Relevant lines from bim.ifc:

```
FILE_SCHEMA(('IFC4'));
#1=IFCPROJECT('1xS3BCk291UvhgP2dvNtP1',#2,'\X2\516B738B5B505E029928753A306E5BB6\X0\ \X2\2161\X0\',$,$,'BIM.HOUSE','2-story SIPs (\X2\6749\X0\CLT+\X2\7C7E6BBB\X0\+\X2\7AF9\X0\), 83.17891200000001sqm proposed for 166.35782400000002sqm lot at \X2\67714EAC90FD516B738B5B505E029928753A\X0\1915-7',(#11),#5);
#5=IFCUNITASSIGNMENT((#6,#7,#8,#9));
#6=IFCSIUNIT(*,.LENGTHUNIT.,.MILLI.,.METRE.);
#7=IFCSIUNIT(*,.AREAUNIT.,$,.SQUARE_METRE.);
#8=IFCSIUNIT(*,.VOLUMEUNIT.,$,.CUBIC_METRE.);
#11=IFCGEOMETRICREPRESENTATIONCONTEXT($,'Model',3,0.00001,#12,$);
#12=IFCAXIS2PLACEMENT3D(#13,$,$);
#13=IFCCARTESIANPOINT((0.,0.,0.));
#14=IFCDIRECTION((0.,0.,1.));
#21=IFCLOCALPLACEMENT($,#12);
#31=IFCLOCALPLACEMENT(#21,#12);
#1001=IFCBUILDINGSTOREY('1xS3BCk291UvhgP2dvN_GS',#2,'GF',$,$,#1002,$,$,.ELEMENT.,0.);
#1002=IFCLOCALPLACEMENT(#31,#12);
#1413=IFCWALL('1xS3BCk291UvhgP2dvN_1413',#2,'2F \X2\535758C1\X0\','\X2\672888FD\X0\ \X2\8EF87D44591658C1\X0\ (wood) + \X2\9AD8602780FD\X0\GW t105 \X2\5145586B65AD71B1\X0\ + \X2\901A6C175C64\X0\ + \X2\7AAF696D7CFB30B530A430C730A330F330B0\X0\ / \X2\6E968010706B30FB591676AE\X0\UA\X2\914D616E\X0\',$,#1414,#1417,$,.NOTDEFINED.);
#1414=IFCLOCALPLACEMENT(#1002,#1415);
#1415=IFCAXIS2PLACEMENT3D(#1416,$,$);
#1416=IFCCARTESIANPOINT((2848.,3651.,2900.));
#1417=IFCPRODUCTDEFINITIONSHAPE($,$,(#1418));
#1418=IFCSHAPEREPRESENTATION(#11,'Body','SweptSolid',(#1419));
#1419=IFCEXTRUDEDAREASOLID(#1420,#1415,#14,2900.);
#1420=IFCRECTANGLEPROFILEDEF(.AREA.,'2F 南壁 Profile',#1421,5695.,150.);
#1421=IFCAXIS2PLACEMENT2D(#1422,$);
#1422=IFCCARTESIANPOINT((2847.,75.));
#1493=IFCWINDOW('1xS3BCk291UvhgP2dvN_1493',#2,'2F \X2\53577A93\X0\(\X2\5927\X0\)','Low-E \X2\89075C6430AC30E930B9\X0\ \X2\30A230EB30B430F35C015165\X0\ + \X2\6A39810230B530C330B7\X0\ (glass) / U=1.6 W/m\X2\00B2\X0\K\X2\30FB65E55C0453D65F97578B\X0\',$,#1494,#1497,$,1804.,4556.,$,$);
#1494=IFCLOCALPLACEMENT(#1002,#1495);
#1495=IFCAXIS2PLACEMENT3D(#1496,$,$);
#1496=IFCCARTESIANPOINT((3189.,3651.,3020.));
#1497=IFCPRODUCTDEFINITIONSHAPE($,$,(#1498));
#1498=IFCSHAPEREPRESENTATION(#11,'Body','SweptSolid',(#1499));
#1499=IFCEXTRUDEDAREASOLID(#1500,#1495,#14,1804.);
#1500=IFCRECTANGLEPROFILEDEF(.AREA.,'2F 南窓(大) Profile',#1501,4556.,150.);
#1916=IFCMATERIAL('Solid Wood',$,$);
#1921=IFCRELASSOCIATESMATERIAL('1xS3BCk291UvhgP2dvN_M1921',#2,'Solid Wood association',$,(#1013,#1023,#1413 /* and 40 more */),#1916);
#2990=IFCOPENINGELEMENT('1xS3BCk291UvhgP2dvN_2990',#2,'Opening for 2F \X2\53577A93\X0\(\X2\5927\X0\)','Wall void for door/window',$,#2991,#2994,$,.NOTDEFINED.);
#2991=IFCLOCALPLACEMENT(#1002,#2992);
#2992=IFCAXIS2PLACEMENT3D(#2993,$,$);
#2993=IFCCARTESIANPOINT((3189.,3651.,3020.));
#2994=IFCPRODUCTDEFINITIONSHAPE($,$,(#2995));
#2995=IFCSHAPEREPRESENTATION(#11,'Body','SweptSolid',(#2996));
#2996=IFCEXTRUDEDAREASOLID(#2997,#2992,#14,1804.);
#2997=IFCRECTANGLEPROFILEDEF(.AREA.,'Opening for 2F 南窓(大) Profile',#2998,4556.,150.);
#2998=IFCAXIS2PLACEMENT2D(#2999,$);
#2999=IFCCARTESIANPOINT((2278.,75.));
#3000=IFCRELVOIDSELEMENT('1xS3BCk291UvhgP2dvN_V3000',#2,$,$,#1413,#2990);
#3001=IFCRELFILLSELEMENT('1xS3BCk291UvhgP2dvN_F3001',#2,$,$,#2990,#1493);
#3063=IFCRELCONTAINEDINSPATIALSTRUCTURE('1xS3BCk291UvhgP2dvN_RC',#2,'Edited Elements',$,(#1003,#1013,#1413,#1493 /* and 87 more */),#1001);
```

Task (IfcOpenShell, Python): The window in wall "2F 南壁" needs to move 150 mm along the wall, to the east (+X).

```python
import ifcopenshell
import ifcopenshell.api.geometry
import ifcopenshell.util.placement
import ifcopenshell.util.unit

model = ifcopenshell.open("bim.ifc")
unit_scale = ifcopenshell.util.unit.calculate_unit_scale(model)

window = model.by_guid("1xS3BCk291UvhgP2dvN_1493")
opening = window.FillsVoids[0].RelatingOpeningElement
wall = opening.VoidsElements[0].RelatingBuildingElement

wall_matrix = ifcopenshell.util.placement.get_local_placement(wall.ObjectPlacement)
shift = wall_matrix[:3, 0] * 0.15 / unit_scale
before = ifcopenshell.util.placement.get_local_placement(window.ObjectPlacement)[:3, 3].copy()

# The window is not placed relative to its opening, so move both.
for product in (opening, window):
    matrix = ifcopenshell.util.placement.get_local_placement(product.ObjectPlacement)
    matrix[:3, 3] += shift
    ifcopenshell.api.geometry.edit_object_placement(model, product=product, matrix=matrix, is_si=False)

after = ifcopenshell.util.placement.get_local_placement(window.ObjectPlacement)[:3, 3]
print("window moved by", (after - before).round(3) + 0.0)

model.write("bim_updated.ifc")
```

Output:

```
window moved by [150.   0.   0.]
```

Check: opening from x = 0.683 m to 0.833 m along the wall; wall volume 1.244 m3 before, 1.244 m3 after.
